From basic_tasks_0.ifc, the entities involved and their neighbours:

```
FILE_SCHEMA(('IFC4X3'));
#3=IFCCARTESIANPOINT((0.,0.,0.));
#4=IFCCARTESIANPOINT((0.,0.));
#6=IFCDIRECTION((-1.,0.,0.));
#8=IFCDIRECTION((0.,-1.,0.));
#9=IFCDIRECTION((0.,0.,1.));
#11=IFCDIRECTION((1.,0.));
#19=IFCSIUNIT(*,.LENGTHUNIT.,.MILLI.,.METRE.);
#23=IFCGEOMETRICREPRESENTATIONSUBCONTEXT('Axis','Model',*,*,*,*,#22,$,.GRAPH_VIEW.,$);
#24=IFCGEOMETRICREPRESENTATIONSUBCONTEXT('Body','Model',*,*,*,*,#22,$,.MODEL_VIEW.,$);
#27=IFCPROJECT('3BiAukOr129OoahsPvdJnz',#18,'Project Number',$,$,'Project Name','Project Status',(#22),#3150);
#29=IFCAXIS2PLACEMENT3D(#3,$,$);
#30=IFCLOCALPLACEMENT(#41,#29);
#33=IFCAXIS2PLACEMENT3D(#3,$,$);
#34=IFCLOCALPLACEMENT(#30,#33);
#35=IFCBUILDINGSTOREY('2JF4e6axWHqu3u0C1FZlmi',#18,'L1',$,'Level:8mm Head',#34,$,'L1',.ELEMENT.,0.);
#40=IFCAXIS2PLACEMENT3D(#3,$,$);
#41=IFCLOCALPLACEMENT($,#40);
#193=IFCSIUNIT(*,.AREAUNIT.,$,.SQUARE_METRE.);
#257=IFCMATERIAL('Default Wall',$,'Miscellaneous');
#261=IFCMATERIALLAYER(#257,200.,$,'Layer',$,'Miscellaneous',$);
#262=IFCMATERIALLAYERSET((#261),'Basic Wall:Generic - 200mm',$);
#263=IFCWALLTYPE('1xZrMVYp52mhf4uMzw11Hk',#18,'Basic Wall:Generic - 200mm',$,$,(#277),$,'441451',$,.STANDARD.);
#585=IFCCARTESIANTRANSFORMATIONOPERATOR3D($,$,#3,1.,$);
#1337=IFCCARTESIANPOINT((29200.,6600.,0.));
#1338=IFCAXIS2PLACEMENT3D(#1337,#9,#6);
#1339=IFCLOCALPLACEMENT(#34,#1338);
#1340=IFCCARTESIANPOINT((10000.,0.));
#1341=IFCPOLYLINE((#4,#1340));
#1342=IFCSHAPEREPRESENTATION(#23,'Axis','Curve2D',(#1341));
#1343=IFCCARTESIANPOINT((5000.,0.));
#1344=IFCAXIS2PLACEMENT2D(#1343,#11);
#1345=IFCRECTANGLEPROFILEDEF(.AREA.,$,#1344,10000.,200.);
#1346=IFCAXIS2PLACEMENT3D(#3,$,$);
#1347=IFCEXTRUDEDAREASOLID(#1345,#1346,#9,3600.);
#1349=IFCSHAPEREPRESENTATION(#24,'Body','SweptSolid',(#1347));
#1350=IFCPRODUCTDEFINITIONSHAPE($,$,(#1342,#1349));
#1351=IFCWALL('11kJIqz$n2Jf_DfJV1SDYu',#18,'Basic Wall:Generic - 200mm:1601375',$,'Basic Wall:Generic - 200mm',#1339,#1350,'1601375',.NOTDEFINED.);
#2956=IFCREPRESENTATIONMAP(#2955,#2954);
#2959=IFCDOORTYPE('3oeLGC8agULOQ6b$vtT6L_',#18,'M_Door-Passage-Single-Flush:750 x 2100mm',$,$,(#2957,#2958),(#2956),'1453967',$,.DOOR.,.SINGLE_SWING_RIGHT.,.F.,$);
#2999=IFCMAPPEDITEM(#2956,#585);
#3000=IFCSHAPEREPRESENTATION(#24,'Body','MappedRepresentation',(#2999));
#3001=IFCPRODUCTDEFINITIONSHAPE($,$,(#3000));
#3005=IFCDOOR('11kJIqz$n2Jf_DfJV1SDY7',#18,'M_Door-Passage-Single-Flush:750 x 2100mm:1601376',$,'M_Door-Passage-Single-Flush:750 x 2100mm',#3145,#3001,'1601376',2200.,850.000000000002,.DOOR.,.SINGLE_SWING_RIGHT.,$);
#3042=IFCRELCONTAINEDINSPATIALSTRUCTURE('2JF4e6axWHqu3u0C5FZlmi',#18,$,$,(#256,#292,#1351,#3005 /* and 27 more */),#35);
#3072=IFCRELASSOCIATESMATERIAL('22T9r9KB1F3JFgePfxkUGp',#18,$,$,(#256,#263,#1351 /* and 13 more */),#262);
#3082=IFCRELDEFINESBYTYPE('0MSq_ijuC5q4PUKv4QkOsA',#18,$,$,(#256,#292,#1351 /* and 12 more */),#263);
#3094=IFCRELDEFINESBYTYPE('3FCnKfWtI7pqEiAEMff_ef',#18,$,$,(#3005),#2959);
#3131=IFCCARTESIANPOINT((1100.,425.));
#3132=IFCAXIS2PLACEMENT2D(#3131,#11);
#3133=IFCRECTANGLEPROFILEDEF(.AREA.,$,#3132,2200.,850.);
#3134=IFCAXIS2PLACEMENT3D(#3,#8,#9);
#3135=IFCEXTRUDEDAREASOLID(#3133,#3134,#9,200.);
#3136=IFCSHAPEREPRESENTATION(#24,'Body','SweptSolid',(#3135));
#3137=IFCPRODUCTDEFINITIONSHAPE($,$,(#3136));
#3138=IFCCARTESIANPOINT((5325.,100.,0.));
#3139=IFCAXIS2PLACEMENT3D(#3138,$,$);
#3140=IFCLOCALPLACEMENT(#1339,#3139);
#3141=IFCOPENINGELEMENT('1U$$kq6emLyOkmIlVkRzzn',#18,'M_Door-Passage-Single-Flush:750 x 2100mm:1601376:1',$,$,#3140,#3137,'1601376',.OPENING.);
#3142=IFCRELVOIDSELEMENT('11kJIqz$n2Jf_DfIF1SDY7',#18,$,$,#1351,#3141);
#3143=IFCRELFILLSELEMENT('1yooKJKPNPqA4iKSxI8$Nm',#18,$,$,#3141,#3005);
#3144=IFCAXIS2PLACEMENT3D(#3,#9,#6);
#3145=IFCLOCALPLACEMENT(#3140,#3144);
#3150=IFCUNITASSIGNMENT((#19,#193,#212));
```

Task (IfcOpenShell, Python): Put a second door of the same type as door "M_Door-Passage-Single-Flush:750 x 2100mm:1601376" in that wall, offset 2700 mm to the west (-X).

```python
import ifcopenshell
import ifcopenshell.api.feature
import ifcopenshell.api.geometry
import ifcopenshell.api.root
import ifcopenshell.geom
import ifcopenshell.util.element
import ifcopenshell.util.placement
import ifcopenshell.util.shape

model = ifcopenshell.open("basic_tasks_0.ifc")
settings = ifcopenshell.geom.settings()


def volume(element):
    """Net volume in cubic metres, openings subtracted."""
    shape = ifcopenshell.geom.create_shape(settings, element)
    return ifcopenshell.util.shape.get_volume(shape.geometry)


def reuse_history(source, copy):
    """copy_class also copies each property set's owner history, people and application; keep the originals."""
    for rel in copy.IsDefinedBy:
        if rel.is_a("IfcRelDefinesByProperties") and (history := rel.RelatingPropertyDefinition.OwnerHistory):
            rel.RelatingPropertyDefinition.OwnerHistory = source.OwnerHistory
            ifcopenshell.util.element.remove_deep2(model, history)


door = model.by_id(3005)
opening = door.FillsVoids[0].RelatingOpeningElement
wall = opening.VoidsElements[0].RelatingBuildingElement
before = volume(wall)
shift = ifcopenshell.util.placement.get_local_placement(wall.ObjectPlacement)[:3, 0] * 2700.0

# copy_class copies the void relationship, type, container and properties, but no geometry.
new_opening = ifcopenshell.api.root.copy_class(model, product=opening)
new_opening.Representation = ifcopenshell.util.element.copy_deep(
    model, opening.Representation, exclude=["IfcGeometricRepresentationContext", "IfcRepresentationMap"]
)
new_opening.Name = "M_Door-Passage-Single-Flush:750 x 2100mm"
new_opening.Tag = None
new_door = ifcopenshell.api.root.copy_class(model, product=door)
new_door.Representation = ifcopenshell.util.element.copy_deep(
    model, door.Representation, exclude=["IfcGeometricRepresentationContext", "IfcRepresentationMap"]
)
new_door.Name = "M_Door-Passage-Single-Flush:750 x 2100mm"
new_door.Tag = None
reuse_history(door, new_door)
ifcopenshell.api.feature.add_filling(model, opening=new_opening, element=new_door)

for old, new in ((opening, new_opening), (door, new_door)):
    matrix = ifcopenshell.util.placement.get_local_placement(old.ObjectPlacement)
    matrix[:3, 3] += shift
    ifcopenshell.api.geometry.edit_object_placement(model, product=new, matrix=matrix, is_si=False)

after = volume(wall)

print(f"wall volume {before:.3f} -> {after:.3f} m3")

model.write("basic_tasks_0_edited.ifc")
```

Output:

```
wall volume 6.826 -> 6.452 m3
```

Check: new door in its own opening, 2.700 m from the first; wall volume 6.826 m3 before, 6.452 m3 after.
